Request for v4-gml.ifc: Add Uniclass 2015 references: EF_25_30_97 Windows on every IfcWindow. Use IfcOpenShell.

First a look at what the model holds.

```python
import ifcopenshell

model = ifcopenshell.open("v4-gml.ifc")
print(model.schema)
print("classifications:", [c.Name for c in model.by_type("IfcClassification")])
for ifc_class in ("IfcDoor", "IfcRoof", "IfcStair", "IfcWall", "IfcWindow"):
    print(ifc_class, len(model.by_type(ifc_class)))
```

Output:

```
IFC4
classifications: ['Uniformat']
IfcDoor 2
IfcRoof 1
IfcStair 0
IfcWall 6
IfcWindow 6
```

```python
import ifcopenshell
import ifcopenshell.api.classification

model = ifcopenshell.open("v4-gml.ifc")

system = ifcopenshell.api.classification.add_classification(model, classification="Uniclass 2015")

codes = {
    "IfcWindow": ("EF_25_30_97", "Windows"),
}
for ifc_class, (code, name) in codes.items():
    products = model.by_type(ifc_class)
    ifcopenshell.api.classification.add_reference(
        model, products=products, classification=system, identification=code, name=name
    )
    print(code, len(products))

model.write("v4-gml_v2.ifc")
```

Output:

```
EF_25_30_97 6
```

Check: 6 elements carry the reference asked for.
